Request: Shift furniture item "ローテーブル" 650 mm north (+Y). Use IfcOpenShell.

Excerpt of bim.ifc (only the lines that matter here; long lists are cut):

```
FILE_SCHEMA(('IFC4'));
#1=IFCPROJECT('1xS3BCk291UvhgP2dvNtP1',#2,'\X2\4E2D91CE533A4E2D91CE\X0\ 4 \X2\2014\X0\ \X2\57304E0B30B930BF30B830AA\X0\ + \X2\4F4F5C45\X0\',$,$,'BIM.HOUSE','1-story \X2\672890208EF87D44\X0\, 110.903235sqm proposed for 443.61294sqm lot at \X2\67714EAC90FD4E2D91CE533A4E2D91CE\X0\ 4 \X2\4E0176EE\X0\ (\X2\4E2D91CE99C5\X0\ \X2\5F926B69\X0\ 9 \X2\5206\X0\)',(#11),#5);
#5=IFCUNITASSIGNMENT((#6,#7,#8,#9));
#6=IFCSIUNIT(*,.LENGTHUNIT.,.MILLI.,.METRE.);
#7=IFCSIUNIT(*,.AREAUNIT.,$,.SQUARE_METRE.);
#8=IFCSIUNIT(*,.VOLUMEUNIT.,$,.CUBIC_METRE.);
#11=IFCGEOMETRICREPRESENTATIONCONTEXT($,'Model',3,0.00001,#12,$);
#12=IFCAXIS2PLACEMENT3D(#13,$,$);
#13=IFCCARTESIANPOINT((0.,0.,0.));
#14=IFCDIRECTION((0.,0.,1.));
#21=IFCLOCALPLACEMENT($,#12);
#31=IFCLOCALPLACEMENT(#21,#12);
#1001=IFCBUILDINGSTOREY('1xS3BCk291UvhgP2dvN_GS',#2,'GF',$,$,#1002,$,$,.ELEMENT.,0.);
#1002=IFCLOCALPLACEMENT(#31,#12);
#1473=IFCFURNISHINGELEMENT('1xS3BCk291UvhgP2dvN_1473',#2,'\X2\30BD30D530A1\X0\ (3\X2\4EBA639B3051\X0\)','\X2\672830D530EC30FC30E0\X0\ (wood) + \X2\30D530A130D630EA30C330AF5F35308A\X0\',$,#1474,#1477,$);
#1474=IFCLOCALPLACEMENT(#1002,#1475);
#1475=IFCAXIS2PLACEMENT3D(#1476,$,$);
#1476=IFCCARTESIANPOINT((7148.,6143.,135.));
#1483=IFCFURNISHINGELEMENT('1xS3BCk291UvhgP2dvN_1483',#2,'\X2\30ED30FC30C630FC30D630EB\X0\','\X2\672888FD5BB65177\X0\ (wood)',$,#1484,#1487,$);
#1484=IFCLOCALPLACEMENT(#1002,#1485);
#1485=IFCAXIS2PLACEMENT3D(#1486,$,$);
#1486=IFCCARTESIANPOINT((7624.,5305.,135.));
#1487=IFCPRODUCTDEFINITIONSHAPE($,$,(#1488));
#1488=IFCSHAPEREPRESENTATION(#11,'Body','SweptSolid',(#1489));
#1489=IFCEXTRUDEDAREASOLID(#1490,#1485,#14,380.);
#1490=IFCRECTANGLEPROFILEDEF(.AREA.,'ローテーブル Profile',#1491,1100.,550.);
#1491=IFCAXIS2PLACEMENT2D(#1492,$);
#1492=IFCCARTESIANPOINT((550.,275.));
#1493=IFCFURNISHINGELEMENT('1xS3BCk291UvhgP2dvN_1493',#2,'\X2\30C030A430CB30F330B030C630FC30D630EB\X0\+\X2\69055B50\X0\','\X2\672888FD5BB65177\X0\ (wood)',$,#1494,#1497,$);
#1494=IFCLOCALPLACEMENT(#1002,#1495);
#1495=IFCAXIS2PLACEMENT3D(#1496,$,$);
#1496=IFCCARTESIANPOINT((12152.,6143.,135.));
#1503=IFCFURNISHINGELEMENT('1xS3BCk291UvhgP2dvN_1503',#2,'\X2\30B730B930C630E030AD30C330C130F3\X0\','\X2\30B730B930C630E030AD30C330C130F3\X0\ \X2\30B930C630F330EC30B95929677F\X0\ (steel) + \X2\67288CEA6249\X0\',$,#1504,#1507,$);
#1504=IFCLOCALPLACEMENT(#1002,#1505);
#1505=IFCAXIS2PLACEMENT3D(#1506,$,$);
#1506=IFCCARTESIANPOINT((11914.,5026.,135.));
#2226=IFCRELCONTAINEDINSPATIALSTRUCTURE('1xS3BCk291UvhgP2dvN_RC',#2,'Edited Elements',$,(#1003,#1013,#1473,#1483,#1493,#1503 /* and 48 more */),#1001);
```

```python
import ifcopenshell
import ifcopenshell.api.geometry
import ifcopenshell.util.placement
import ifcopenshell.util.unit

model = ifcopenshell.open("bim.ifc")
unit_scale = ifcopenshell.util.unit.calculate_unit_scale(model)

item = model.by_guid("1xS3BCk291UvhgP2dvN_1483")
matrix = ifcopenshell.util.placement.get_local_placement(item.ObjectPlacement)
matrix[1, 3] += 0.65 / unit_scale
ifcopenshell.api.geometry.edit_object_placement(model, product=item, matrix=matrix, is_si=False)

print(ifcopenshell.util.placement.get_local_placement(item.ObjectPlacement).round(3) + 0.0)

model.write("bim_v2.ifc")
```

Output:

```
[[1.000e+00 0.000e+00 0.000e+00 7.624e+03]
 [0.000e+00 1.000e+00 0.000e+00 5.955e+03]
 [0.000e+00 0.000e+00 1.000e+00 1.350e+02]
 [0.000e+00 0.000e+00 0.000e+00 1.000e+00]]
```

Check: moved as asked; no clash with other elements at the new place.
